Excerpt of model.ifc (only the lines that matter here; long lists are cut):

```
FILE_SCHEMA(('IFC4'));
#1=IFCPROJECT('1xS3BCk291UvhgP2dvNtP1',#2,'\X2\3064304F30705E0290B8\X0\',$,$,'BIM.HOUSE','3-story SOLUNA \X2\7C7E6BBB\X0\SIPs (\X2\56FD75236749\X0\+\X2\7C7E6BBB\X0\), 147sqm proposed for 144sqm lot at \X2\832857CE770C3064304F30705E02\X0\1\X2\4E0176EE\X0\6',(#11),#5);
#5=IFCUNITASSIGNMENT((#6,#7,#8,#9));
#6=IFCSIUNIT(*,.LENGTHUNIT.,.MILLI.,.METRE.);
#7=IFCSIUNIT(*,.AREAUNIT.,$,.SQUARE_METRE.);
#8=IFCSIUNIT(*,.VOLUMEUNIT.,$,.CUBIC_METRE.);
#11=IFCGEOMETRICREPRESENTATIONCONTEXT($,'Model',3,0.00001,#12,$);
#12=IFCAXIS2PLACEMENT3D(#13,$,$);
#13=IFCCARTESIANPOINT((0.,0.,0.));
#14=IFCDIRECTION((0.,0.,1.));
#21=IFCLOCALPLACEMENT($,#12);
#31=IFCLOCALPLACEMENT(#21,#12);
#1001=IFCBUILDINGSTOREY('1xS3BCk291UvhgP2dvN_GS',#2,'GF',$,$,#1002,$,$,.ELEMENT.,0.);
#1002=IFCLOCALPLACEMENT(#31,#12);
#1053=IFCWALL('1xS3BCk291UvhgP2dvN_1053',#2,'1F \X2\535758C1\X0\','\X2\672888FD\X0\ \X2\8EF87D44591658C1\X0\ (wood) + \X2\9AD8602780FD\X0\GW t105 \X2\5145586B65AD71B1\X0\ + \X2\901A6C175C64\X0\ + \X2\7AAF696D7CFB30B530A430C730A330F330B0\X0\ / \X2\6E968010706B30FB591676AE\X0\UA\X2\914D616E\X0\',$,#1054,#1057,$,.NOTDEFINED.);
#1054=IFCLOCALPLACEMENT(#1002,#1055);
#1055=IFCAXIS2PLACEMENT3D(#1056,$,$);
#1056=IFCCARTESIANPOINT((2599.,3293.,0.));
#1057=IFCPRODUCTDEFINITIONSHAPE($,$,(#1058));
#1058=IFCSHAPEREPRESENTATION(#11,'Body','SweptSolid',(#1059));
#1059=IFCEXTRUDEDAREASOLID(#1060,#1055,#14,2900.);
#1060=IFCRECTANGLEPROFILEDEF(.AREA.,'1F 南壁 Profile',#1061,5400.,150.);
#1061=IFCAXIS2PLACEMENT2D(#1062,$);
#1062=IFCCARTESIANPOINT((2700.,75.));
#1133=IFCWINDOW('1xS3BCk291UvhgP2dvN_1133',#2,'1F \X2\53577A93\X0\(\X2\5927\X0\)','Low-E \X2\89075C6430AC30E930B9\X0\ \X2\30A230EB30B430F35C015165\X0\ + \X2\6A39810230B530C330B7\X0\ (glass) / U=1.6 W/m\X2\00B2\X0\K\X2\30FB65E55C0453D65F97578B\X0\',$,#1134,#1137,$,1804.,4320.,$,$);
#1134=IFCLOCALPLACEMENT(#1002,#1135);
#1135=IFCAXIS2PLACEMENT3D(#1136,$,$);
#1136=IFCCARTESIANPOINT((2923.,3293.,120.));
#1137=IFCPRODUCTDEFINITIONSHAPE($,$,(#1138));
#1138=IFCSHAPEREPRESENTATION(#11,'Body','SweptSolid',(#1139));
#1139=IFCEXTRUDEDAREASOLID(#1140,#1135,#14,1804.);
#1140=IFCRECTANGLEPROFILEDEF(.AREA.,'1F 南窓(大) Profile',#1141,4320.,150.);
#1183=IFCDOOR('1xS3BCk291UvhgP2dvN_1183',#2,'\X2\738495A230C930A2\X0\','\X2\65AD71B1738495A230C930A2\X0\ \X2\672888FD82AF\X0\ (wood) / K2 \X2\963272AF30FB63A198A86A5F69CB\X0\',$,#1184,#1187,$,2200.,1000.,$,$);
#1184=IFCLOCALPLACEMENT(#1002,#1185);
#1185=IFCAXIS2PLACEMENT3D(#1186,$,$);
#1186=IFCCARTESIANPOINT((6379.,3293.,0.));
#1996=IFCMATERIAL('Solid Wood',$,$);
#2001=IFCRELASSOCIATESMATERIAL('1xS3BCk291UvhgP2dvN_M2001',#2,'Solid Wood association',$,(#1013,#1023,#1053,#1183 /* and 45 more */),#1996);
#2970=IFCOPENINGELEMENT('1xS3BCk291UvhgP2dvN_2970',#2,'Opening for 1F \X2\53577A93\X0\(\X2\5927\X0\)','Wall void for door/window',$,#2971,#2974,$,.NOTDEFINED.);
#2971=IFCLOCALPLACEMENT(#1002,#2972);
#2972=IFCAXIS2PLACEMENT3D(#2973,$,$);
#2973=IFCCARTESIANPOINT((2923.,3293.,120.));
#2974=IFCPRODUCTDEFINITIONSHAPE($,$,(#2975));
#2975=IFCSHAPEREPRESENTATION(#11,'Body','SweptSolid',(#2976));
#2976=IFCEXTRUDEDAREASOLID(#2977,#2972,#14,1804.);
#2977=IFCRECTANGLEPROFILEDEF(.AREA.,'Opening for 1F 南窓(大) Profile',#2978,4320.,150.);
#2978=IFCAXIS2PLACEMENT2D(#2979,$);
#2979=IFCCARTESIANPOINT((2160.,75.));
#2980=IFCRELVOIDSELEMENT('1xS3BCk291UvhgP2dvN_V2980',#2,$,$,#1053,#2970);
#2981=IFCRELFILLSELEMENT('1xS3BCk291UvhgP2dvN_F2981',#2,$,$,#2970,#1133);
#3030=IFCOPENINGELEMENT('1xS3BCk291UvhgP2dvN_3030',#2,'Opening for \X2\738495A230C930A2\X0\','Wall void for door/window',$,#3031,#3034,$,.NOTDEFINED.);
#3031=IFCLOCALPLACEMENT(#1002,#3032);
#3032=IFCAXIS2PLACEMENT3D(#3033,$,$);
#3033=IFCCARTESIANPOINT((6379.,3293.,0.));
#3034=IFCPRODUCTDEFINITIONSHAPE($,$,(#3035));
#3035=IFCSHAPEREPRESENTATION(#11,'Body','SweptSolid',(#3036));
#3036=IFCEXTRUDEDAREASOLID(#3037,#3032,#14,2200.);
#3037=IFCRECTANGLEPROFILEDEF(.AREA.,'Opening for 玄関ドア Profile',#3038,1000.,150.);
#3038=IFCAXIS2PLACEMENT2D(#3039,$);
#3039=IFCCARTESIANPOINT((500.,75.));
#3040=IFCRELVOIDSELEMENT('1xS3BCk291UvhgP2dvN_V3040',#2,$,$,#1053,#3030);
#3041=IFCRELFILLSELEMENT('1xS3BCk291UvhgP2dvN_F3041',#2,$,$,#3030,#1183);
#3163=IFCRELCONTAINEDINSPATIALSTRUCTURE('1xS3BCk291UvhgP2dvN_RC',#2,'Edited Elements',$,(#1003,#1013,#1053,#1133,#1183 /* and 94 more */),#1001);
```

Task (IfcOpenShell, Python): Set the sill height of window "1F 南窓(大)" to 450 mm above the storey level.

```python
import numpy as np
import ifcopenshell
import ifcopenshell.api.geometry
import ifcopenshell.geom
import ifcopenshell.util.element
import ifcopenshell.util.placement
import ifcopenshell.util.shape
import ifcopenshell.util.unit

model = ifcopenshell.open("model.ifc")
unit_scale = ifcopenshell.util.unit.calculate_unit_scale(model)

window = model.by_id(1133)
opening = window.FillsVoids[0].RelatingOpeningElement
storey = ifcopenshell.util.element.get_container(window, ifc_class="IfcBuildingStorey")
level = ifcopenshell.util.placement.get_local_placement(storey.ObjectPlacement)[2, 3]

# The opening's origin need not be at the sill, so measure its lowest point.
shape = ifcopenshell.geom.create_shape(ifcopenshell.geom.settings(), opening)
bottom = ifcopenshell.util.shape.get_shape_bottom_elevation(shape, shape.geometry) / unit_scale
dz = level + 450.0 - bottom

shift = np.array([0.0, 0.0, dz])
# The window is not placed relative to its opening, so move both.
for product in (opening, window):
    matrix = ifcopenshell.util.placement.get_local_placement(product.ObjectPlacement)
    matrix[:3, 3] += shift
    ifcopenshell.api.geometry.edit_object_placement(model, product=product, matrix=matrix, is_si=False)

print(f"moved by {dz * unit_scale:+.3f} m")

model.write("model_edited.ifc")
```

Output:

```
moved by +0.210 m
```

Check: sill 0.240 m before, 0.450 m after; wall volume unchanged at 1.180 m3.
